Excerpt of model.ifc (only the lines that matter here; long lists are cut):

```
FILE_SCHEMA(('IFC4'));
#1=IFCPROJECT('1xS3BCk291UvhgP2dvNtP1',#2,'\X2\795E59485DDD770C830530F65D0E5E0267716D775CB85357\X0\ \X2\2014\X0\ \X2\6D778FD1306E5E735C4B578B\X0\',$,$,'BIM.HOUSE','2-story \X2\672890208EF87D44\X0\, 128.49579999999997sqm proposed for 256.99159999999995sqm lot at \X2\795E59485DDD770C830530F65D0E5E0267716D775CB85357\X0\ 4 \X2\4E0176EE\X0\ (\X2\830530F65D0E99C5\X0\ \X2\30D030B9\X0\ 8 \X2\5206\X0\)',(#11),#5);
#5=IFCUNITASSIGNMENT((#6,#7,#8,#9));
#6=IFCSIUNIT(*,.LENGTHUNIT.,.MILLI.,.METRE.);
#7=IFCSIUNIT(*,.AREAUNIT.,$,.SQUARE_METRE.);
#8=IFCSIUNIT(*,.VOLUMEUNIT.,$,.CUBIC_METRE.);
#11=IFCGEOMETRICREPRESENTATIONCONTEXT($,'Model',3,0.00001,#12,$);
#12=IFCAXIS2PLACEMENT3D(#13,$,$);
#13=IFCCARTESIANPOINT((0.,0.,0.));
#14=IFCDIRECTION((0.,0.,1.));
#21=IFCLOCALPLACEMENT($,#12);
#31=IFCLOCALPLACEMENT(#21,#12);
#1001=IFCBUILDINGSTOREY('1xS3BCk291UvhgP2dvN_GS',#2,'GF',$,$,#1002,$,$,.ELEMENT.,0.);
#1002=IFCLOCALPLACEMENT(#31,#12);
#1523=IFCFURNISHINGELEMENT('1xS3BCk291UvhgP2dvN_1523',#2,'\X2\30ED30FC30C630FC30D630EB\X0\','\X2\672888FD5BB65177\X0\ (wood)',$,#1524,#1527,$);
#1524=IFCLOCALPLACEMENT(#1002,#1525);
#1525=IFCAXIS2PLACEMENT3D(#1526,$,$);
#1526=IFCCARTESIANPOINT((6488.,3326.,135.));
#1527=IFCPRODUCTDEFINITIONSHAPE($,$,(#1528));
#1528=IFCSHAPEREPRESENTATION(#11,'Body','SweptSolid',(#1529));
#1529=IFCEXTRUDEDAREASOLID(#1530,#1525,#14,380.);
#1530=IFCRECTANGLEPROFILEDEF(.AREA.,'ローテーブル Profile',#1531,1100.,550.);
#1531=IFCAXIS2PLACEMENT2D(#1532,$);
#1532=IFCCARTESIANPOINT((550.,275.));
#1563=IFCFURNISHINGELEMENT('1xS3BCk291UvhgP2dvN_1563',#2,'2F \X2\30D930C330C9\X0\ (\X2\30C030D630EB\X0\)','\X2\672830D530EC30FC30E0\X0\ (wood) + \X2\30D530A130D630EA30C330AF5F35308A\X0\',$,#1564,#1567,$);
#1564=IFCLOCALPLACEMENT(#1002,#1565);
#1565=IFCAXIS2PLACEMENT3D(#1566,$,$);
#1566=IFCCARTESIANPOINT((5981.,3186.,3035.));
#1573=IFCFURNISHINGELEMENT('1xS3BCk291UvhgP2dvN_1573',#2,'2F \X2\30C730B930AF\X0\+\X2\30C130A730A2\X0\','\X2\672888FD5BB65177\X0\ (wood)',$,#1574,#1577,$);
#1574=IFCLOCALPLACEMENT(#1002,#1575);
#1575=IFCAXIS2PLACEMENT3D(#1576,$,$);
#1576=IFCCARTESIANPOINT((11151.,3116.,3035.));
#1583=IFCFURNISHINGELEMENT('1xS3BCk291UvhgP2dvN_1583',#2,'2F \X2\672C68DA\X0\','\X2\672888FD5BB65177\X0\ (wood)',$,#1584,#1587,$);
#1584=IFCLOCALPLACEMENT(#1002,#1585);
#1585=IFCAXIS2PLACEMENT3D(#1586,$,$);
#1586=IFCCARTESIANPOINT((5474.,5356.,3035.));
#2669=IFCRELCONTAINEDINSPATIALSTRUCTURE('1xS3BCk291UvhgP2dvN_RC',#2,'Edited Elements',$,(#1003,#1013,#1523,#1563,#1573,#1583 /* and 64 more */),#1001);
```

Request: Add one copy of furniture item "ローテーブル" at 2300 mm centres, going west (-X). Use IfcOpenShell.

```python
import numpy as np
import ifcopenshell
import ifcopenshell.api.geometry
import ifcopenshell.api.root
import ifcopenshell.util.element
import ifcopenshell.util.placement

model = ifcopenshell.open("model.ifc")


def reuse_history(source, copy):
    """copy_class also copies each property set's owner history, people and application; keep the originals."""
    for rel in copy.IsDefinedBy:
        if rel.is_a("IfcRelDefinesByProperties") and (history := rel.RelatingPropertyDefinition.OwnerHistory):
            rel.RelatingPropertyDefinition.OwnerHistory = source.OwnerHistory
            ifcopenshell.util.element.remove_deep2(model, history)


source = model.by_guid("1xS3BCk291UvhgP2dvN_1523")
base = ifcopenshell.util.placement.get_local_placement(source.ObjectPlacement)
step = np.array([-1.0, 0.0, 0.0]) * 2300.0

for i in range(1, 2):
    copy = ifcopenshell.api.root.copy_class(model, product=source)
    copy.Representation = ifcopenshell.util.element.copy_deep(
        model, source.Representation, exclude=["IfcGeometricRepresentationContext", "IfcRepresentationMap"]
    )
    reuse_history(source, copy)
    matrix = base.copy()
    matrix[:3, 3] += i * step
    print("added at", matrix[:3, 3].round(3) + 0.0)
    ifcopenshell.api.geometry.edit_object_placement(model, product=copy, matrix=matrix, is_si=False)

model.write("model_rev.ifc")
```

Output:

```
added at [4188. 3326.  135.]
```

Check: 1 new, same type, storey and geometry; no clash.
